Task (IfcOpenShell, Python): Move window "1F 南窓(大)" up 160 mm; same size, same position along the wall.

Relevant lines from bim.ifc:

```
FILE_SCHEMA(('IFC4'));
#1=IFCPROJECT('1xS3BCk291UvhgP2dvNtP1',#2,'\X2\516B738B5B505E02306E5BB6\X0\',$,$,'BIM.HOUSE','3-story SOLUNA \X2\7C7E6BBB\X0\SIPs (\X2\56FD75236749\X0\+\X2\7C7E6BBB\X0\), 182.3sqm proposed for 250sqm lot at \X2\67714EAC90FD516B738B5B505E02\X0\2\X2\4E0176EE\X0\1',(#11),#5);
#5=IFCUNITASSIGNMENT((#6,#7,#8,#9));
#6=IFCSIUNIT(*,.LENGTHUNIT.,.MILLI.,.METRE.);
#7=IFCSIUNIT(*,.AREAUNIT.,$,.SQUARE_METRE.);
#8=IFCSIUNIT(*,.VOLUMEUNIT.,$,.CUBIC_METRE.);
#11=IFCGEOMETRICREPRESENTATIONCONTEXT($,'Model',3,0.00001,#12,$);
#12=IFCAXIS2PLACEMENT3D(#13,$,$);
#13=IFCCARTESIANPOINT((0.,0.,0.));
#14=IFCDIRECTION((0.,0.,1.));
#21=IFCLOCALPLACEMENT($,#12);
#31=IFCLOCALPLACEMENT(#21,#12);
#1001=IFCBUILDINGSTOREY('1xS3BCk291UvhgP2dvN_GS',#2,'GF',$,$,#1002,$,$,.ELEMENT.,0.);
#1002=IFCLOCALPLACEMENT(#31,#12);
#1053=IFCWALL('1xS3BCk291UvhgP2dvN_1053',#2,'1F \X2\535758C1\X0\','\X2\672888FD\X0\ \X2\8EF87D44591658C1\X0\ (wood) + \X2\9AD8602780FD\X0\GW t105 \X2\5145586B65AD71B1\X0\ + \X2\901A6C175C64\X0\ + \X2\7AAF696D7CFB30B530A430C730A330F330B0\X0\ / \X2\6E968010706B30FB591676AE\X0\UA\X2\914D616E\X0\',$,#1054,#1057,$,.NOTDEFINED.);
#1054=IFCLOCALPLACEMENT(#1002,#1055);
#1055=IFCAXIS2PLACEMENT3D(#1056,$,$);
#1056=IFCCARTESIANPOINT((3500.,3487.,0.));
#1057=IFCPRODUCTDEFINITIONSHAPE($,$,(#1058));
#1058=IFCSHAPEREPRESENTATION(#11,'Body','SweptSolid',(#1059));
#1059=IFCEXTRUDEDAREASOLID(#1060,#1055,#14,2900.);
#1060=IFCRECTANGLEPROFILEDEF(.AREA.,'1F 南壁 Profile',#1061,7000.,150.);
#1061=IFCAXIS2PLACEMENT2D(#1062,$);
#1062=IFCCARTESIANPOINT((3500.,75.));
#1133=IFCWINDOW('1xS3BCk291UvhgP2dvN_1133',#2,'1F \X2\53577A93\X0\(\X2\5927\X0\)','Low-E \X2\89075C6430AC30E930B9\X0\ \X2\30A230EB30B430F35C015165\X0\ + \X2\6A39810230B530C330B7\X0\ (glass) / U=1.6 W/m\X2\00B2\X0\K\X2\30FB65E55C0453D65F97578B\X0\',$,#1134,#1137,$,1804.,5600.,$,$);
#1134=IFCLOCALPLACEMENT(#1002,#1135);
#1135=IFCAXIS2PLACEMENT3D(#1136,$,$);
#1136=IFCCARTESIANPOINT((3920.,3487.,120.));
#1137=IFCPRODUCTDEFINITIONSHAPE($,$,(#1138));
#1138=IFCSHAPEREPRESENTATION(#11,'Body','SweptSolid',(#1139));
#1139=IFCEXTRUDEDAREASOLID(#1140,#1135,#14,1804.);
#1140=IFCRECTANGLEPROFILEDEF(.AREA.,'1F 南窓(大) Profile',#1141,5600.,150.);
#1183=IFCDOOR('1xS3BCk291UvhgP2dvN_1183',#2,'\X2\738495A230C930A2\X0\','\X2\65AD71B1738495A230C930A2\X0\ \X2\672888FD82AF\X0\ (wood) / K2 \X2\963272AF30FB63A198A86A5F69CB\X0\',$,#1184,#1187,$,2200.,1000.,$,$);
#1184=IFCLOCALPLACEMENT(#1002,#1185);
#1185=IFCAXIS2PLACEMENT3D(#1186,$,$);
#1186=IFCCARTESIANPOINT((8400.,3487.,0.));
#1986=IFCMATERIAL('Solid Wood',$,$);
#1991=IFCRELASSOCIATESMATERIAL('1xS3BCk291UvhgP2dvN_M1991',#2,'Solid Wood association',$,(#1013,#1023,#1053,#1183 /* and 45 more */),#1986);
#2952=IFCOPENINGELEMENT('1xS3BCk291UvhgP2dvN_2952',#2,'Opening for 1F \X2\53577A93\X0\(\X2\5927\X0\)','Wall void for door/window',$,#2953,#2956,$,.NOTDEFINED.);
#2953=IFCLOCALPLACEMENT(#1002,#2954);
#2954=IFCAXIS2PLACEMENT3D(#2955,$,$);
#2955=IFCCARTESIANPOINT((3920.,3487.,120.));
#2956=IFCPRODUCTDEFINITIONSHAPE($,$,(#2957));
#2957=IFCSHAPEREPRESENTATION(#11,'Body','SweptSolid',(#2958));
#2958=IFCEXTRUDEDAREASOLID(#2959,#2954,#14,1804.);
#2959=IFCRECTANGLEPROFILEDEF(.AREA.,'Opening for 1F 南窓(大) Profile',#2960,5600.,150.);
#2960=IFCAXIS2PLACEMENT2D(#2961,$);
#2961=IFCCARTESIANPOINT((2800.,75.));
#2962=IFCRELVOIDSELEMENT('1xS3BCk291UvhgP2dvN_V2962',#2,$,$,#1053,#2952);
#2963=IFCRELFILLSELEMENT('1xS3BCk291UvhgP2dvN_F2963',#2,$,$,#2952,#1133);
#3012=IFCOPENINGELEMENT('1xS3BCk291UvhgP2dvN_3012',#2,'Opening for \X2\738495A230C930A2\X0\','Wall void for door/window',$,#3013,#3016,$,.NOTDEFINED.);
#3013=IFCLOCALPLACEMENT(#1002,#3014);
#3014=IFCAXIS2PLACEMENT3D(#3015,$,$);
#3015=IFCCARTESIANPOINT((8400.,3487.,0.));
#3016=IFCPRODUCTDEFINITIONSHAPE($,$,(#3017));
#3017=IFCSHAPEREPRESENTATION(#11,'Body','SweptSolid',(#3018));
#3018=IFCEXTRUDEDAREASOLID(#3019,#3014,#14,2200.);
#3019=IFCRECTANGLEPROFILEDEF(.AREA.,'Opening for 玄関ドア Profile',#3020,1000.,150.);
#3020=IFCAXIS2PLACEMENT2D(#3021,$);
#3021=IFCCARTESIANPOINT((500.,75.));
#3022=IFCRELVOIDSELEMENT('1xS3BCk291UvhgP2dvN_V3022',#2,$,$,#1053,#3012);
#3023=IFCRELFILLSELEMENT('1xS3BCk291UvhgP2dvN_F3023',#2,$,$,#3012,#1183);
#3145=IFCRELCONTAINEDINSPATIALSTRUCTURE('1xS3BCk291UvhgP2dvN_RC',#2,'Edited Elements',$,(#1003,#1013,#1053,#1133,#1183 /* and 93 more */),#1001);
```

```python
import numpy as np
import ifcopenshell
import ifcopenshell.api.geometry
import ifcopenshell.util.placement
import ifcopenshell.util.unit

model = ifcopenshell.open("bim.ifc")
unit_scale = ifcopenshell.util.unit.calculate_unit_scale(model)

window = model.by_id(1133)
opening = window.FillsVoids[0].RelatingOpeningElement
dz = 0.16 / unit_scale

shift = np.array([0.0, 0.0, dz])
# The window is not placed relative to its opening, so move both.
for product in (opening, window):
    matrix = ifcopenshell.util.placement.get_local_placement(product.ObjectPlacement)
    matrix[:3, 3] += shift
    ifcopenshell.api.geometry.edit_object_placement(model, product=product, matrix=matrix, is_si=False)

print(f"moved by {dz * unit_scale:+.3f} m")

model.write("bim_edited.ifc")
```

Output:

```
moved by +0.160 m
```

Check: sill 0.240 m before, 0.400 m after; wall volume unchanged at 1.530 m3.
